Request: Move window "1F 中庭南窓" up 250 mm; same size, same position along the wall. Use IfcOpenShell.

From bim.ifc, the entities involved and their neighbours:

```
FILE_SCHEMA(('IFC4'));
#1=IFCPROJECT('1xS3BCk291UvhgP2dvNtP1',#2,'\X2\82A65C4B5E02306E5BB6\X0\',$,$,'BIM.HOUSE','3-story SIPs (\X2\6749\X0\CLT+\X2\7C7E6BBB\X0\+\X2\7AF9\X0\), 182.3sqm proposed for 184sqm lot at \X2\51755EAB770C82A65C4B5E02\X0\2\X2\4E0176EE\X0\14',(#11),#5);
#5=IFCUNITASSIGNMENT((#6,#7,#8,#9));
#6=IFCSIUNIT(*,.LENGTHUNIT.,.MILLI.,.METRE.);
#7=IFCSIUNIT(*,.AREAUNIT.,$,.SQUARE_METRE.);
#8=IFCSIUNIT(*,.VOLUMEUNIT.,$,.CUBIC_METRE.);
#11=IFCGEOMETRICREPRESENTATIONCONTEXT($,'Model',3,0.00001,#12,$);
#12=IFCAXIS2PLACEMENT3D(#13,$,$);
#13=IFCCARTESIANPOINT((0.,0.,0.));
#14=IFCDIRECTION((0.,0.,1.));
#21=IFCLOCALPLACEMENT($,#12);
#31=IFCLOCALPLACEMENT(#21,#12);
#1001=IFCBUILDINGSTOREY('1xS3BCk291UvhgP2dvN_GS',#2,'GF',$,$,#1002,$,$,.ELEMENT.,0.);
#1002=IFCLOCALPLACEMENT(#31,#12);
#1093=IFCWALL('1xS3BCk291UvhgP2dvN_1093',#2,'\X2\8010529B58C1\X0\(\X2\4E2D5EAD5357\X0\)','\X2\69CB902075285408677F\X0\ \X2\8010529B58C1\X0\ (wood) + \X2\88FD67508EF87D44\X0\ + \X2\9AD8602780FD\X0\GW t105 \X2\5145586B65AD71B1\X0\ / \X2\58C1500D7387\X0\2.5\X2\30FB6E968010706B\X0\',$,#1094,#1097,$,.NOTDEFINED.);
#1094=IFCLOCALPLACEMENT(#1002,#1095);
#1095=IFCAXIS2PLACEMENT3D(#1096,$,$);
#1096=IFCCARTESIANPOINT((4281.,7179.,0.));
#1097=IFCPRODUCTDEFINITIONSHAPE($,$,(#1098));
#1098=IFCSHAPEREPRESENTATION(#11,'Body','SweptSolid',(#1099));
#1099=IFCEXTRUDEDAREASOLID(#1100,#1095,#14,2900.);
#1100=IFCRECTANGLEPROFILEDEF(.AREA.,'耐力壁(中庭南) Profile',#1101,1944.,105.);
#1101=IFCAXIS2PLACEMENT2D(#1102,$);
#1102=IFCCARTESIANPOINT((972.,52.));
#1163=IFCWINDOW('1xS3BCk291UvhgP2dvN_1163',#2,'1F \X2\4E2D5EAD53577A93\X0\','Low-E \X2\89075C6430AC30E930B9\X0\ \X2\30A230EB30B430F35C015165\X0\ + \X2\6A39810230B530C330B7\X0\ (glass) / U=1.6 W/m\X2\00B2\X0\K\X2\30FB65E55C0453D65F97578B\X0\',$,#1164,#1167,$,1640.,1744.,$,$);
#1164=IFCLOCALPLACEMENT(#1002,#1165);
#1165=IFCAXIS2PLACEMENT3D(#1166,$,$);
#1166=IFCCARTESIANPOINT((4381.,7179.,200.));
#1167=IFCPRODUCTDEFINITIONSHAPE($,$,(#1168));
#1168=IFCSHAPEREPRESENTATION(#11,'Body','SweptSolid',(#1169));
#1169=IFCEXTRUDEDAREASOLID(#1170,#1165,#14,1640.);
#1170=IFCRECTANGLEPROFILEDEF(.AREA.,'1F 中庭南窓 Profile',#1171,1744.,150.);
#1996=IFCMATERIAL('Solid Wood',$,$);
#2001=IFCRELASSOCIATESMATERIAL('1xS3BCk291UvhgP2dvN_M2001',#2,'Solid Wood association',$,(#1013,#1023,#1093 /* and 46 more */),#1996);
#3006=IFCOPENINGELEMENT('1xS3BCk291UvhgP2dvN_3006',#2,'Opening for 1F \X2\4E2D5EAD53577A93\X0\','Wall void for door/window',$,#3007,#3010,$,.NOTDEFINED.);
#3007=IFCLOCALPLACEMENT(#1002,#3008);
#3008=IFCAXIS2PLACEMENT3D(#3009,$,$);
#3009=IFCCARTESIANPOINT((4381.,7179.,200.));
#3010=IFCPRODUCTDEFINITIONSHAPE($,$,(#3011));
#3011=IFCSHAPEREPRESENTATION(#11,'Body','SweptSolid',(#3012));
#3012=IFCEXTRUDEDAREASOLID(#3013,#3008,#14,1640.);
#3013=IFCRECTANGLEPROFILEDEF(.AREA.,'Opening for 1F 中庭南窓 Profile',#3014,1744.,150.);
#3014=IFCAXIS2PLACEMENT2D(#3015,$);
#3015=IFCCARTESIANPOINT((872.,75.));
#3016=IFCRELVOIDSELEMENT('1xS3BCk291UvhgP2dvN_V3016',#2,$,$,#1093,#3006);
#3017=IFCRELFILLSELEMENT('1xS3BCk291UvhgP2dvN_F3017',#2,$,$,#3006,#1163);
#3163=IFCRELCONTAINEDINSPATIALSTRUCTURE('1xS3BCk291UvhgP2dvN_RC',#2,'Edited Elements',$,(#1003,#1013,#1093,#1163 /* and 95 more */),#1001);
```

```python
import numpy as np
import ifcopenshell
import ifcopenshell.api.geometry
import ifcopenshell.util.placement
import ifcopenshell.util.unit

model = ifcopenshell.open("bim.ifc")
unit_scale = ifcopenshell.util.unit.calculate_unit_scale(model)

window = model.by_guid("1xS3BCk291UvhgP2dvN_1163")
opening = window.FillsVoids[0].RelatingOpeningElement
dz = 250.0

shift = np.array([0.0, 0.0, dz])
# The window is not placed relative to its opening, so move both.
for product in (opening, window):
    matrix = ifcopenshell.util.placement.get_local_placement(product.ObjectPlacement)
    matrix[:3, 3] += shift
    ifcopenshell.api.geometry.edit_object_placement(model, product=product, matrix=matrix, is_si=False)

print(f"moved by {dz * unit_scale:+.3f} m")

model.write("bim_updated.ifc")
```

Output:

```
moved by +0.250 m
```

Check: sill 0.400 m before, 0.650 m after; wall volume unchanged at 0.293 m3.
